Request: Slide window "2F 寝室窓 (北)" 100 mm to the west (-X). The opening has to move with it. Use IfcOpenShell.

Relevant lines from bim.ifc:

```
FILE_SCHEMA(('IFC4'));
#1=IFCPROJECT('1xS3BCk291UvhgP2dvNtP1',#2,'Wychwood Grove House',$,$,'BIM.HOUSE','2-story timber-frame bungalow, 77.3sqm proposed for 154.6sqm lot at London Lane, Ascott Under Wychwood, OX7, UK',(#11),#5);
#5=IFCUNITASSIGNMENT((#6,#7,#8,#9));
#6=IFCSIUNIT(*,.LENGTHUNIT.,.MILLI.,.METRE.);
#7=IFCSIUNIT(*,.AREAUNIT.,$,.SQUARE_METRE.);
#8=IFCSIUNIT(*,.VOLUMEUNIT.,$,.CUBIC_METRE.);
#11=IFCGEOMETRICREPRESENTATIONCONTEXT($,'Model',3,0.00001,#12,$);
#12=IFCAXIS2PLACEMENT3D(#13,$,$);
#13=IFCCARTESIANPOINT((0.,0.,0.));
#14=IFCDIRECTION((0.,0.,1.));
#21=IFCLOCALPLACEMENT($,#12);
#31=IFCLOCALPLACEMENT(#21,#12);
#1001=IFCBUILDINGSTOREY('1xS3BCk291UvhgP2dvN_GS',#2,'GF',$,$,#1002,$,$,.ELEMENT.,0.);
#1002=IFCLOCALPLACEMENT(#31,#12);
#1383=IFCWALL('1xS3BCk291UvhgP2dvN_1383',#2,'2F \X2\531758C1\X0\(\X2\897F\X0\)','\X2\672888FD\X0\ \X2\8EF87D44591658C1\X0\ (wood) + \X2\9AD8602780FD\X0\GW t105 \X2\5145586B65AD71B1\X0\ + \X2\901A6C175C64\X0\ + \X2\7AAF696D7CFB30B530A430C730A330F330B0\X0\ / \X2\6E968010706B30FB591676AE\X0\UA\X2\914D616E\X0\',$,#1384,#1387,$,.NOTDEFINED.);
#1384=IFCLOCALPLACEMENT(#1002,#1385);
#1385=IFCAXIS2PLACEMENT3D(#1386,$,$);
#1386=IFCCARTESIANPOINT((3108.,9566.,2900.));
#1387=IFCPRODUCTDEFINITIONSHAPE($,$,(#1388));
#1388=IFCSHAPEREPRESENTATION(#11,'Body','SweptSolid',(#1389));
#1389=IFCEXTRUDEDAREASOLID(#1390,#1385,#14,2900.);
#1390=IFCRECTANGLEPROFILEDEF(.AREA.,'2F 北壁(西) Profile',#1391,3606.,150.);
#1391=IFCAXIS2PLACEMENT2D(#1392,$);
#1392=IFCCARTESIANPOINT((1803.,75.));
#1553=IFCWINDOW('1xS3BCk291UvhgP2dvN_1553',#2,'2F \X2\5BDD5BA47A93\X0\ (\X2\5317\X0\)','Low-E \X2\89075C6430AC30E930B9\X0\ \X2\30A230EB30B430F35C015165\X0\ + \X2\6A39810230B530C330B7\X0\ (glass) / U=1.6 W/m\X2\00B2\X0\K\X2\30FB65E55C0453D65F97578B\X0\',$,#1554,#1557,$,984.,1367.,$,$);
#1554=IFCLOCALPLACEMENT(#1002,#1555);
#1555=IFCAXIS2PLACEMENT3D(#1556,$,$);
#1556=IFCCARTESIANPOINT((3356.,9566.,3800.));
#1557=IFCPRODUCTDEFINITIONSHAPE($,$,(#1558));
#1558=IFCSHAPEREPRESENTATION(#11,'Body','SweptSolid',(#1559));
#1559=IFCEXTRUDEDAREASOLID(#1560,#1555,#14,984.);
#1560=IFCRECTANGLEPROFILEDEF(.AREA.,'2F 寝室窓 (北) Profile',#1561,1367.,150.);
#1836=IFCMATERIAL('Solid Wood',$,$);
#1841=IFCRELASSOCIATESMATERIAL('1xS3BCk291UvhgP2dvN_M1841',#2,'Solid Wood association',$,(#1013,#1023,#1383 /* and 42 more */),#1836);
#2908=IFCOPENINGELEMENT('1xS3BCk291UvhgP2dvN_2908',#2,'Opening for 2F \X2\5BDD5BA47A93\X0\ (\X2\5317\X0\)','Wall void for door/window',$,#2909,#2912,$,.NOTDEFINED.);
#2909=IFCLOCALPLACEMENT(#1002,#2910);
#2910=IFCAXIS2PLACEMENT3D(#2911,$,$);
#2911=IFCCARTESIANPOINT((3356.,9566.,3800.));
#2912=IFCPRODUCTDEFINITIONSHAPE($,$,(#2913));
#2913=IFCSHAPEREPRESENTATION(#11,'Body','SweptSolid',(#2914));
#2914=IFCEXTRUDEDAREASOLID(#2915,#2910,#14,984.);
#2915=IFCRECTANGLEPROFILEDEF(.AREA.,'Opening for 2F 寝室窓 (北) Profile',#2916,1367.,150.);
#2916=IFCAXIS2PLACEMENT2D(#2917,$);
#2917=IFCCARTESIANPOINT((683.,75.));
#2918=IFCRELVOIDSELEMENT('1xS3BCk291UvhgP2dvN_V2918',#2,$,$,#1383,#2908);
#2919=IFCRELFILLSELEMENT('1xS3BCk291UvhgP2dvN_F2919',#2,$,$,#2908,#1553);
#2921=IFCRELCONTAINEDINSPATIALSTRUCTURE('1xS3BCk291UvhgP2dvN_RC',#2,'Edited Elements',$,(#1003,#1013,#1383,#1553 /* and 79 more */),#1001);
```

```python
import ifcopenshell
import ifcopenshell.api.geometry
import ifcopenshell.util.placement
import ifcopenshell.util.unit

model = ifcopenshell.open("bim.ifc")
unit_scale = ifcopenshell.util.unit.calculate_unit_scale(model)

window = model.by_id(1553)
opening = window.FillsVoids[0].RelatingOpeningElement
wall = opening.VoidsElements[0].RelatingBuildingElement

wall_matrix = ifcopenshell.util.placement.get_local_placement(wall.ObjectPlacement)
shift = wall_matrix[:3, 0] * -0.1 / unit_scale
before = ifcopenshell.util.placement.get_local_placement(window.ObjectPlacement)[:3, 3].copy()

# The window is not placed relative to its opening, so move both.
for product in (opening, window):
    matrix = ifcopenshell.util.placement.get_local_placement(product.ObjectPlacement)
    matrix[:3, 3] += shift
    ifcopenshell.api.geometry.edit_object_placement(model, product=product, matrix=matrix, is_si=False)

after = ifcopenshell.util.placement.get_local_placement(window.ObjectPlacement)[:3, 3]
print("window moved by", (after - before).round(3) + 0.0)

model.write("bim-out.ifc")
```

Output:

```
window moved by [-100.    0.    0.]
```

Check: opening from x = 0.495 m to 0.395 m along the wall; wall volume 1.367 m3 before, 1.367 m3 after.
